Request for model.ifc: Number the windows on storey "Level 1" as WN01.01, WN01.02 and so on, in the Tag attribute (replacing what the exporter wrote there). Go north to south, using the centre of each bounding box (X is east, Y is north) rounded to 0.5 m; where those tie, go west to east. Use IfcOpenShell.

First a look at what the model holds.

```python
import ifcopenshell
import ifcopenshell.util.element
import ifcopenshell.util.placement

model = ifcopenshell.open("model.ifc")
print(model.schema)
storey = next(s for s in model.by_type("IfcBuildingStorey") if s.Name == "Level 1")
windows = [e for e in ifcopenshell.util.element.get_decomposition(storey) if e.is_a("IfcWindow")]
for e in sorted(windows, key=lambda e: e.id()):
    origin = ifcopenshell.util.placement.get_local_placement(e.ObjectPlacement)[:3, 3]
    print(e.id(), e.Tag, e.Name, origin.round(2) + 0.0, sep=" | ")
```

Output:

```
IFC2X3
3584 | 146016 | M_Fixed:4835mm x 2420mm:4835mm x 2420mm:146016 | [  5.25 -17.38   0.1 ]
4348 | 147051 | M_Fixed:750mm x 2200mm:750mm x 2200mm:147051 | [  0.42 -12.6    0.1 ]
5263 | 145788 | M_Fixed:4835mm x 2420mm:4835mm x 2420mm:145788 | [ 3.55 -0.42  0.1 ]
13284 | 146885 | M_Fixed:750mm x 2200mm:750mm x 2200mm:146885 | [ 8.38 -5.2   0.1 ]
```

```python
import ifcopenshell
import ifcopenshell.geom
import ifcopenshell.util.element
import ifcopenshell.util.shape

model = ifcopenshell.open("model.ifc")
settings = ifcopenshell.geom.settings()
settings.set("use-world-coords", True)


def centre(element):
    shape = ifcopenshell.geom.create_shape(settings, element)
    return ifcopenshell.util.shape.get_bbox_centroid(shape.geometry)


storey = next(s for s in model.by_type("IfcBuildingStorey") if s.Name == "Level 1")
windows = [e for e in ifcopenshell.util.element.get_decomposition(storey) if e.is_a("IfcWindow")]

# Insertion points can sit at a corner or the storey origin, so sort by the geometry (in metres).
centres = {e: centre(e) for e in windows}
windows.sort(key=lambda e: (-round(centres[e][1] / 0.5), centres[e][0]))

for i, e in enumerate(windows, start=1):
    number = f"WN01.{i:02d}"
    e.Tag = number
    print(e.id(), number)

model.write("model_edited.ifc")
```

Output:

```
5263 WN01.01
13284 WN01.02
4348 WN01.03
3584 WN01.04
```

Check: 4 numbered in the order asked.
